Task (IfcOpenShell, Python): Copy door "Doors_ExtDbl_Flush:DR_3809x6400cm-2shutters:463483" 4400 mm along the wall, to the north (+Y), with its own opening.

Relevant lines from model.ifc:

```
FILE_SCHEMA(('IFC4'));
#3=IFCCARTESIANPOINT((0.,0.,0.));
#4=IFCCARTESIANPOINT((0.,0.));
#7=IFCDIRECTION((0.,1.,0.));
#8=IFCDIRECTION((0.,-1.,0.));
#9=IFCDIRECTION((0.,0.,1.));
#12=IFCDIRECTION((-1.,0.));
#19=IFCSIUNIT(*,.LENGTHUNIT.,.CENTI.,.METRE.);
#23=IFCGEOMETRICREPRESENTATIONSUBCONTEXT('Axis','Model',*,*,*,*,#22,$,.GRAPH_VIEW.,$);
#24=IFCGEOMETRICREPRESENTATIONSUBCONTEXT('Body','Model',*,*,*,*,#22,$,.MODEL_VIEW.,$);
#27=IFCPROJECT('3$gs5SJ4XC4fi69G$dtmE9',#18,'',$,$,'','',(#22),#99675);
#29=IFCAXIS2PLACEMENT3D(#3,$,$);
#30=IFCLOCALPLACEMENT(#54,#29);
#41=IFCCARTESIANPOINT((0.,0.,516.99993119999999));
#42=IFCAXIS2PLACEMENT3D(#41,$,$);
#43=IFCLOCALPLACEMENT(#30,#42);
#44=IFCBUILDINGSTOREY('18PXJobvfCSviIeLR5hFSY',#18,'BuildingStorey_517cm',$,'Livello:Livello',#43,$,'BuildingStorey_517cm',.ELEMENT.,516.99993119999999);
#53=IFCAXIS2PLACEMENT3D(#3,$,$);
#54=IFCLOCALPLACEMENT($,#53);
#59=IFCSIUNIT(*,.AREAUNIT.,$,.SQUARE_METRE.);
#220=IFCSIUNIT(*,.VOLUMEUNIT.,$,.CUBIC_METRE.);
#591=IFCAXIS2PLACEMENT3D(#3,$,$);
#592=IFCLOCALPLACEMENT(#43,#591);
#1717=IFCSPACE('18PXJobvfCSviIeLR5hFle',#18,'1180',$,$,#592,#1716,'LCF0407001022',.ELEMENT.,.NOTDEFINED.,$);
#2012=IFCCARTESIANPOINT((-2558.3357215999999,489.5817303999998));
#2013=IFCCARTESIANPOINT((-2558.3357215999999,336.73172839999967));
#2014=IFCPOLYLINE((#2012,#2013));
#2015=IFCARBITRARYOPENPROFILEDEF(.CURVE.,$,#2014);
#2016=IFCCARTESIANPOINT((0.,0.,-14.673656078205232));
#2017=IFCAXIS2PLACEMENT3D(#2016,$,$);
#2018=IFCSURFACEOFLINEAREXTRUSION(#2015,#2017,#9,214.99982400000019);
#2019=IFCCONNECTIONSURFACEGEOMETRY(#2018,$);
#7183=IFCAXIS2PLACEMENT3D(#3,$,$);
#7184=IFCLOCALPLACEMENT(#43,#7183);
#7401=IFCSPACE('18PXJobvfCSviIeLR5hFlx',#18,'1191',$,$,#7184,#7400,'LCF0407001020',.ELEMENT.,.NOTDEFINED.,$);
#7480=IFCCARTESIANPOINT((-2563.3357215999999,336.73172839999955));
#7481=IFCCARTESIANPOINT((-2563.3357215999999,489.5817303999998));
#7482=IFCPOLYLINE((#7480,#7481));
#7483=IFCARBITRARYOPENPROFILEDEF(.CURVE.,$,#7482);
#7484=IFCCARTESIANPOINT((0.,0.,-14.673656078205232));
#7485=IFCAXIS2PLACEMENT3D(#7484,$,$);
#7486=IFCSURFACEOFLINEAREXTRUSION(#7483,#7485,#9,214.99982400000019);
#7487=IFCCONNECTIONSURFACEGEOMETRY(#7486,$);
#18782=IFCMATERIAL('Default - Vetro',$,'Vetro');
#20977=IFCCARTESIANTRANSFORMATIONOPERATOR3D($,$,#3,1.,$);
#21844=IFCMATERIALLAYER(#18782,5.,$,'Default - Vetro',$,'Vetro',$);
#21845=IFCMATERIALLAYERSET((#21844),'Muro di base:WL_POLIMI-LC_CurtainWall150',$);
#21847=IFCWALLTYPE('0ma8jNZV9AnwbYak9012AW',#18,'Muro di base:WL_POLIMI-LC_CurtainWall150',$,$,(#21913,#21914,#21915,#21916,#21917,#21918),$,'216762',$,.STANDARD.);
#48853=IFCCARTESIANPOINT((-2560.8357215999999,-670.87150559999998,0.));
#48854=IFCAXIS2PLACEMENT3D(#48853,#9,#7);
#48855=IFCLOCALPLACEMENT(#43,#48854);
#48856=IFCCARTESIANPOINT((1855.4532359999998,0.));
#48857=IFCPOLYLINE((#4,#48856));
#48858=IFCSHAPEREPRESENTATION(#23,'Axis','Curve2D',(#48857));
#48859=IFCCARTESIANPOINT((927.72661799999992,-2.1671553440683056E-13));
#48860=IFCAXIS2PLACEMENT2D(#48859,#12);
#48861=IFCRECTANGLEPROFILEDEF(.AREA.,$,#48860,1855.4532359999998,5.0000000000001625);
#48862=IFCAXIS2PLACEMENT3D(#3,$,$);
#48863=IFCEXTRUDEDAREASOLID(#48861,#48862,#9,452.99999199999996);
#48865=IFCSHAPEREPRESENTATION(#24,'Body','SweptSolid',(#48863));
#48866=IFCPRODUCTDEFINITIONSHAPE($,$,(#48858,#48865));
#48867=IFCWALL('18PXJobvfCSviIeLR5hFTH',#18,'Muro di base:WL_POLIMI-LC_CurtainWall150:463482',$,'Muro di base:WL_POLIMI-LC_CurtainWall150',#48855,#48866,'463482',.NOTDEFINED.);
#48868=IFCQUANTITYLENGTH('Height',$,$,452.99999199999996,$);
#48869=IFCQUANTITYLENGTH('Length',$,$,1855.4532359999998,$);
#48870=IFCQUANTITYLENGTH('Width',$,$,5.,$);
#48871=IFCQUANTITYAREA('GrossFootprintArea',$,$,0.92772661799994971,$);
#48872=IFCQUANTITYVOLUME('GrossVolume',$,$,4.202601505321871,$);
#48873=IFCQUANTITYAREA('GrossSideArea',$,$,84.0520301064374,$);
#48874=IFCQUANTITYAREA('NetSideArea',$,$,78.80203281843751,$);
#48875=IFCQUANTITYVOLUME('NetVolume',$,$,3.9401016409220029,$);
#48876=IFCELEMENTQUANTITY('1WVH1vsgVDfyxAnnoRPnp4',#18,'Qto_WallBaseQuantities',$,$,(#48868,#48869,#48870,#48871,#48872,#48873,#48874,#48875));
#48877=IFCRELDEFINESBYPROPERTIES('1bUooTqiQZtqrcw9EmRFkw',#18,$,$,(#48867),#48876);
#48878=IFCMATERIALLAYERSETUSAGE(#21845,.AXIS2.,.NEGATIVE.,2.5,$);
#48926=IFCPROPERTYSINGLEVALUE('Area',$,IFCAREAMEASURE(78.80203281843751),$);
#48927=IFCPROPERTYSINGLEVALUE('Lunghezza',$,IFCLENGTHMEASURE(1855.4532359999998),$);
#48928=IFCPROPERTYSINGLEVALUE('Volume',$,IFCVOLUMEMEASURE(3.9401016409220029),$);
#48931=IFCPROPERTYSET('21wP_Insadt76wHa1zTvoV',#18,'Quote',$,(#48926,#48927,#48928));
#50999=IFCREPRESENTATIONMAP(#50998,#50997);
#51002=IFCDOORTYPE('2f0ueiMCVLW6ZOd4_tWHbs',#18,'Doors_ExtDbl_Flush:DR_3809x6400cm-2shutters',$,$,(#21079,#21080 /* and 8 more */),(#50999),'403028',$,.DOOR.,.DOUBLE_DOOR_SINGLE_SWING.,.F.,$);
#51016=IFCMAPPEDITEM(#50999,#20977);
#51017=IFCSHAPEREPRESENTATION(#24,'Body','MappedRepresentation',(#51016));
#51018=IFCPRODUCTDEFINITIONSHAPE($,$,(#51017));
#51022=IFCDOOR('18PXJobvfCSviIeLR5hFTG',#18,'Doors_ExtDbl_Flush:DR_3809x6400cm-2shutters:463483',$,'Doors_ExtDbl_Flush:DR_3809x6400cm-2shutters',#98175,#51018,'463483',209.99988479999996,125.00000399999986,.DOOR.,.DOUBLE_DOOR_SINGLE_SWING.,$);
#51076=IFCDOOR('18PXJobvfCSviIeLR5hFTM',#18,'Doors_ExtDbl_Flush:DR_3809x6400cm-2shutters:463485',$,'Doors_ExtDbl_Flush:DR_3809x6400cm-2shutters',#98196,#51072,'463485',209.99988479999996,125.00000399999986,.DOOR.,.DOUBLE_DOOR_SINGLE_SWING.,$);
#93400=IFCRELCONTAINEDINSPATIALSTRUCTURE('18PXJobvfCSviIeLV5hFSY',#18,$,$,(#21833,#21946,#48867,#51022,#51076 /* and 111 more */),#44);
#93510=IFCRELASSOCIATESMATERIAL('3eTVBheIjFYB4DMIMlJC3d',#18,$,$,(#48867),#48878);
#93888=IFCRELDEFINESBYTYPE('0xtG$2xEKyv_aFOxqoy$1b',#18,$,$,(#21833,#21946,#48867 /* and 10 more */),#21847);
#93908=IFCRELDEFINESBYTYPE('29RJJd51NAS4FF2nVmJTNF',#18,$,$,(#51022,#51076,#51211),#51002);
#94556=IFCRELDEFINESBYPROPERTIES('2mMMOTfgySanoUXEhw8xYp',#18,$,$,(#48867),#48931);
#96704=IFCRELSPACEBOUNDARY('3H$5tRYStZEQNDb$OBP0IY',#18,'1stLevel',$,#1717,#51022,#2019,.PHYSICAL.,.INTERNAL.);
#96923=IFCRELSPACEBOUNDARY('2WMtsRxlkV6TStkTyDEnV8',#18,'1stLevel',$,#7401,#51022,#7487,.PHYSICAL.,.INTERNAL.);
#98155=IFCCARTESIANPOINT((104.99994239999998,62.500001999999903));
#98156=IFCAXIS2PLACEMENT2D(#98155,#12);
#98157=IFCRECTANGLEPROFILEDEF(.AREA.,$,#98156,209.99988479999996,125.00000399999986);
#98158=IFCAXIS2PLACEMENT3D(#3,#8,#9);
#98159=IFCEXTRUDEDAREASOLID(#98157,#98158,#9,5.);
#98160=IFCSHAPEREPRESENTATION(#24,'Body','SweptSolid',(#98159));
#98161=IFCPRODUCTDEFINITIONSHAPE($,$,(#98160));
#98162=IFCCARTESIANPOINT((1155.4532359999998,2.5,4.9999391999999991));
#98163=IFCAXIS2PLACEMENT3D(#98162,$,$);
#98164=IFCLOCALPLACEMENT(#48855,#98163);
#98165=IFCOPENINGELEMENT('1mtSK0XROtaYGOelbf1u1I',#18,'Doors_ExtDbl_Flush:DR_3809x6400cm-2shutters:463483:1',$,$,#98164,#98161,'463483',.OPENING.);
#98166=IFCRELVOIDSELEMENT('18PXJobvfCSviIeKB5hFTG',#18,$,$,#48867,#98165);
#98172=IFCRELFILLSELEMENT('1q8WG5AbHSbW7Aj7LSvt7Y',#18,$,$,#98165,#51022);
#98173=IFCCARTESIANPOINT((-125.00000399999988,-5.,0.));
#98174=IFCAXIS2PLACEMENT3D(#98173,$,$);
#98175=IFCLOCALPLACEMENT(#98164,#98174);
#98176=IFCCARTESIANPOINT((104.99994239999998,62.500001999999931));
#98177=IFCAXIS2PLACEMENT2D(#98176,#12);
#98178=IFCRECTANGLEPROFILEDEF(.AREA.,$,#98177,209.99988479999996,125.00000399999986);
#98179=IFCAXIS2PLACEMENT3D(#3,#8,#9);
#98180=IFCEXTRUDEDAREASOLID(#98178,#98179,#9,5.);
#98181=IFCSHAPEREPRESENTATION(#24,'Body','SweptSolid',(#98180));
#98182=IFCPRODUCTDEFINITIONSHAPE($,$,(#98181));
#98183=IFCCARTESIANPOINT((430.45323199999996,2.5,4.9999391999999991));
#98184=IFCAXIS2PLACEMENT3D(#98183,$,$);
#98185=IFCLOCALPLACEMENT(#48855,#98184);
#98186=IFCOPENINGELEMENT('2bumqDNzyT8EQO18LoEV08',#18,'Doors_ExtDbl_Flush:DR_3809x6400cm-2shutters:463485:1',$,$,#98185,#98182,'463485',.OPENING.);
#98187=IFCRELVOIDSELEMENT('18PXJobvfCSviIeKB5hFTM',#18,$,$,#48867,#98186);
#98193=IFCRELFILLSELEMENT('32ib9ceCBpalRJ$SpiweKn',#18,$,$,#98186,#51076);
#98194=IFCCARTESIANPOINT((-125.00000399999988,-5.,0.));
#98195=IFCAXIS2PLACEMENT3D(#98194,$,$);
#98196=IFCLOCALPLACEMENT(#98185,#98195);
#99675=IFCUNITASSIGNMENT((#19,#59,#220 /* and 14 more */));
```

```python
import numpy as np
import ifcopenshell
import ifcopenshell.api.feature
import ifcopenshell.api.geometry
import ifcopenshell.api.pset
import ifcopenshell.api.root
import ifcopenshell.geom
import ifcopenshell.util.element
import ifcopenshell.util.placement
import ifcopenshell.util.shape
import ifcopenshell.util.unit

model = ifcopenshell.open("model.ifc")
unit_scale = ifcopenshell.util.unit.calculate_unit_scale(model)
area_scale = ifcopenshell.util.unit.calculate_unit_scale(model, "AREAUNIT")
volume_scale = ifcopenshell.util.unit.calculate_unit_scale(model, "VOLUMEUNIT")
settings = ifcopenshell.geom.settings()


def volume(element):
    """Net volume in cubic metres, openings subtracted."""
    shape = ifcopenshell.geom.create_shape(settings, element)
    return ifcopenshell.util.shape.get_volume(shape.geometry)


def reuse_history(source, copy):
    """copy_class also copies each property set's owner history, people and application; keep the originals."""
    for rel in copy.IsDefinedBy:
        if rel.is_a("IfcRelDefinesByProperties") and (history := rel.RelatingPropertyDefinition.OwnerHistory):
            rel.RelatingPropertyDefinition.OwnerHistory = source.OwnerHistory
            ifcopenshell.util.element.remove_deep2(model, history)


door = model.by_guid("18PXJobvfCSviIeLR5hFTG")
opening = door.FillsVoids[0].RelatingOpeningElement
wall = opening.VoidsElements[0].RelatingBuildingElement
before = volume(wall)
shift = ifcopenshell.util.placement.get_local_placement(wall.ObjectPlacement)[:3, 0] * 4.4 / unit_scale

# copy_class copies the void relationship, type, container and properties, but no geometry.
new_opening = ifcopenshell.api.root.copy_class(model, product=opening)
new_opening.Representation = ifcopenshell.util.element.copy_deep(
    model, opening.Representation, exclude=["IfcGeometricRepresentationContext", "IfcRepresentationMap"]
)
new_opening.Name = "Doors_ExtDbl_Flush:DR_3809x6400cm-2shutters"
new_opening.Tag = None
reuse_history(opening, new_opening)
new_door = ifcopenshell.api.root.copy_class(model, product=door)
new_door.Representation = ifcopenshell.util.element.copy_deep(
    model, door.Representation, exclude=["IfcGeometricRepresentationContext", "IfcRepresentationMap"]
)
new_door.Name = "Doors_ExtDbl_Flush:DR_3809x6400cm-2shutters"
new_door.Tag = None
reuse_history(door, new_door)
ifcopenshell.api.feature.add_filling(model, opening=new_opening, element=new_door)

for old, new in ((opening, new_opening), (door, new_door)):
    matrix = ifcopenshell.util.placement.get_local_placement(old.ObjectPlacement)
    matrix[:3, 3] += shift
    ifcopenshell.api.geometry.edit_object_placement(model, product=new, matrix=matrix, is_si=False)

# The copied space boundaries still share their surfaces with the original.
for rel in new_door.ProvidesBoundaries:
    if rel.ConnectionGeometry:
        rel.ConnectionGeometry = ifcopenshell.util.element.copy_deep(model, rel.ConnectionGeometry)

# Space boundary surfaces are stored in each space's coordinates; move them too.
for rel in new_door.ProvidesBoundaries:
    if not rel.ConnectionGeometry:
        continue
    surface = rel.ConnectionGeometry.SurfaceOnRelatingElement
    space_matrix = ifcopenshell.util.placement.get_local_placement(rel.RelatingSpace.ObjectPlacement)
    point = np.array(surface.Position.Location.Coordinates) + space_matrix[:3, :3].T @ shift
    surface.Position = model.createIfcAxis2Placement3D(
        model.createIfcCartesianPoint(point.tolist()), surface.Position.Axis, surface.Position.RefDirection
    )

after = volume(wall)
thickness = 0.05  # wall thickness in metres

# Update the wall's stored quantities.
qto = model.by_id(ifcopenshell.util.element.get_pset(wall, "Qto_WallBaseQuantities", should_inherit=False)["id"])
ifcopenshell.api.pset.edit_qto(model, qto=qto, properties={
    "NetSideArea": after / thickness / area_scale,
    "NetVolume": after / volume_scale,
})
pset = model.by_id(ifcopenshell.util.element.get_pset(wall, "Quote", should_inherit=False)["id"])
ifcopenshell.api.pset.edit_pset(model, pset=pset, properties={
    "Area": model.create_entity("IfcAreaMeasure", after / thickness / area_scale),
    "Volume": model.create_entity("IfcVolumeMeasure", after / volume_scale),
})

print(f"wall volume {before:.3f} -> {after:.3f} m3")

model.write("model-out.ifc")
```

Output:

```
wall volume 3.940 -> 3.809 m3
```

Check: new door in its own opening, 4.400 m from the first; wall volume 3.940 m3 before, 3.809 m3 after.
